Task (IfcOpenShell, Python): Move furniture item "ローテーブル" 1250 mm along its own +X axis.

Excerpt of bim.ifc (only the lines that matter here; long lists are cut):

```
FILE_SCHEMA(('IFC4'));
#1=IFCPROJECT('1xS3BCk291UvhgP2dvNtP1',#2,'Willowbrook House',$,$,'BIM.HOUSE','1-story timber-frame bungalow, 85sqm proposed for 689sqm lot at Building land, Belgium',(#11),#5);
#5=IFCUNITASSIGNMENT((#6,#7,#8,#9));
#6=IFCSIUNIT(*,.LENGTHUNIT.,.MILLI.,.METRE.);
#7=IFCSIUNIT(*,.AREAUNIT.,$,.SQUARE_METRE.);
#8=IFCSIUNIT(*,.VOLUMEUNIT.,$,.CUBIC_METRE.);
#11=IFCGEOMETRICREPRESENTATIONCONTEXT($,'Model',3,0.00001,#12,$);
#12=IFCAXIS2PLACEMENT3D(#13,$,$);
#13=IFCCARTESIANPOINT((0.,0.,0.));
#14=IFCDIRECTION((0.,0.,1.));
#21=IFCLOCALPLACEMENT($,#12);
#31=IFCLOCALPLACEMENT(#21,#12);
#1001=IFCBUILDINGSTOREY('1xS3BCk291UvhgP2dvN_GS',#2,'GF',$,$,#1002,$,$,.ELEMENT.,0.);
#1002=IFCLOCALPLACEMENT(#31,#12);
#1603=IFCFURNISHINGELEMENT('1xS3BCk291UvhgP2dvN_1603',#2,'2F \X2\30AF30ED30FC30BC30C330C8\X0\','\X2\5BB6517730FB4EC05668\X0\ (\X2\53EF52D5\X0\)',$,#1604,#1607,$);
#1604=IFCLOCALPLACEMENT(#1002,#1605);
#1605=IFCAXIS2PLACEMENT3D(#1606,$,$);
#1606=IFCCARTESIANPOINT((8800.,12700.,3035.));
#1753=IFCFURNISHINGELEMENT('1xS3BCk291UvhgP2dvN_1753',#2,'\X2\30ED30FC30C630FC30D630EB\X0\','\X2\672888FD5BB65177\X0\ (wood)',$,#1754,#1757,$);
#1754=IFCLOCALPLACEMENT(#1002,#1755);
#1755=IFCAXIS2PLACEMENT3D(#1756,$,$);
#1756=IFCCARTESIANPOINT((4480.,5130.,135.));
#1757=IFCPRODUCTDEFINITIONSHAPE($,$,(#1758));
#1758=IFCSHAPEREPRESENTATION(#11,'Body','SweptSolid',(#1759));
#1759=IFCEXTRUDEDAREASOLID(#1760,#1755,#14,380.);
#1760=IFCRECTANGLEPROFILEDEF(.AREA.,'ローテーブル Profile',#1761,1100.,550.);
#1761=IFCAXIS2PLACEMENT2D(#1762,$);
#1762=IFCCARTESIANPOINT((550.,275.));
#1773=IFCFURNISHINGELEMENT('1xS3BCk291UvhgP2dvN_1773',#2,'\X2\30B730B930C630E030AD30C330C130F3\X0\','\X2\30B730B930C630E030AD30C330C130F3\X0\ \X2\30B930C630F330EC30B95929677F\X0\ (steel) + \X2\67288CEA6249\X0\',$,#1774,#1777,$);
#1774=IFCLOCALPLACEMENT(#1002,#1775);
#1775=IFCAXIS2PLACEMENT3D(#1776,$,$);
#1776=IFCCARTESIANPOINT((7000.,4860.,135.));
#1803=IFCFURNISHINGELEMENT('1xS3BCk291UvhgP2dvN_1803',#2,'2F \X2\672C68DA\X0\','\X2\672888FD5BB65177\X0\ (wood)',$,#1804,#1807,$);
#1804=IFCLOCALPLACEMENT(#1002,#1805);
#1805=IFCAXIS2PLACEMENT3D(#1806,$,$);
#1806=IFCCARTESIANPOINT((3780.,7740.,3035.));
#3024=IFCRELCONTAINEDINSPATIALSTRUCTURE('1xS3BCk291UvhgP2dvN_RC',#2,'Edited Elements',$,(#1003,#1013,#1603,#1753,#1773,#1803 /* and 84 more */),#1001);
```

```python
import ifcopenshell
import ifcopenshell.api.geometry
import ifcopenshell.util.placement
import ifcopenshell.util.unit

model = ifcopenshell.open("bim.ifc")
unit_scale = ifcopenshell.util.unit.calculate_unit_scale(model)

item = model.by_guid("1xS3BCk291UvhgP2dvN_1753")
matrix = ifcopenshell.util.placement.get_local_placement(item.ObjectPlacement)
matrix[:3, 3] += matrix[:3, 0] * 1.25 / unit_scale
ifcopenshell.api.geometry.edit_object_placement(model, product=item, matrix=matrix, is_si=False)

print(ifcopenshell.util.placement.get_local_placement(item.ObjectPlacement).round(3) + 0.0)

model.write("bim_edited.ifc")
```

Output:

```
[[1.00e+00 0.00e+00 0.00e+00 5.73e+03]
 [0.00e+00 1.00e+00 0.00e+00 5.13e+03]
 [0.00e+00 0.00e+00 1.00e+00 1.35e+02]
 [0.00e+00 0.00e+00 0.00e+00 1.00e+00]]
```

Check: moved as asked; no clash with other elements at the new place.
